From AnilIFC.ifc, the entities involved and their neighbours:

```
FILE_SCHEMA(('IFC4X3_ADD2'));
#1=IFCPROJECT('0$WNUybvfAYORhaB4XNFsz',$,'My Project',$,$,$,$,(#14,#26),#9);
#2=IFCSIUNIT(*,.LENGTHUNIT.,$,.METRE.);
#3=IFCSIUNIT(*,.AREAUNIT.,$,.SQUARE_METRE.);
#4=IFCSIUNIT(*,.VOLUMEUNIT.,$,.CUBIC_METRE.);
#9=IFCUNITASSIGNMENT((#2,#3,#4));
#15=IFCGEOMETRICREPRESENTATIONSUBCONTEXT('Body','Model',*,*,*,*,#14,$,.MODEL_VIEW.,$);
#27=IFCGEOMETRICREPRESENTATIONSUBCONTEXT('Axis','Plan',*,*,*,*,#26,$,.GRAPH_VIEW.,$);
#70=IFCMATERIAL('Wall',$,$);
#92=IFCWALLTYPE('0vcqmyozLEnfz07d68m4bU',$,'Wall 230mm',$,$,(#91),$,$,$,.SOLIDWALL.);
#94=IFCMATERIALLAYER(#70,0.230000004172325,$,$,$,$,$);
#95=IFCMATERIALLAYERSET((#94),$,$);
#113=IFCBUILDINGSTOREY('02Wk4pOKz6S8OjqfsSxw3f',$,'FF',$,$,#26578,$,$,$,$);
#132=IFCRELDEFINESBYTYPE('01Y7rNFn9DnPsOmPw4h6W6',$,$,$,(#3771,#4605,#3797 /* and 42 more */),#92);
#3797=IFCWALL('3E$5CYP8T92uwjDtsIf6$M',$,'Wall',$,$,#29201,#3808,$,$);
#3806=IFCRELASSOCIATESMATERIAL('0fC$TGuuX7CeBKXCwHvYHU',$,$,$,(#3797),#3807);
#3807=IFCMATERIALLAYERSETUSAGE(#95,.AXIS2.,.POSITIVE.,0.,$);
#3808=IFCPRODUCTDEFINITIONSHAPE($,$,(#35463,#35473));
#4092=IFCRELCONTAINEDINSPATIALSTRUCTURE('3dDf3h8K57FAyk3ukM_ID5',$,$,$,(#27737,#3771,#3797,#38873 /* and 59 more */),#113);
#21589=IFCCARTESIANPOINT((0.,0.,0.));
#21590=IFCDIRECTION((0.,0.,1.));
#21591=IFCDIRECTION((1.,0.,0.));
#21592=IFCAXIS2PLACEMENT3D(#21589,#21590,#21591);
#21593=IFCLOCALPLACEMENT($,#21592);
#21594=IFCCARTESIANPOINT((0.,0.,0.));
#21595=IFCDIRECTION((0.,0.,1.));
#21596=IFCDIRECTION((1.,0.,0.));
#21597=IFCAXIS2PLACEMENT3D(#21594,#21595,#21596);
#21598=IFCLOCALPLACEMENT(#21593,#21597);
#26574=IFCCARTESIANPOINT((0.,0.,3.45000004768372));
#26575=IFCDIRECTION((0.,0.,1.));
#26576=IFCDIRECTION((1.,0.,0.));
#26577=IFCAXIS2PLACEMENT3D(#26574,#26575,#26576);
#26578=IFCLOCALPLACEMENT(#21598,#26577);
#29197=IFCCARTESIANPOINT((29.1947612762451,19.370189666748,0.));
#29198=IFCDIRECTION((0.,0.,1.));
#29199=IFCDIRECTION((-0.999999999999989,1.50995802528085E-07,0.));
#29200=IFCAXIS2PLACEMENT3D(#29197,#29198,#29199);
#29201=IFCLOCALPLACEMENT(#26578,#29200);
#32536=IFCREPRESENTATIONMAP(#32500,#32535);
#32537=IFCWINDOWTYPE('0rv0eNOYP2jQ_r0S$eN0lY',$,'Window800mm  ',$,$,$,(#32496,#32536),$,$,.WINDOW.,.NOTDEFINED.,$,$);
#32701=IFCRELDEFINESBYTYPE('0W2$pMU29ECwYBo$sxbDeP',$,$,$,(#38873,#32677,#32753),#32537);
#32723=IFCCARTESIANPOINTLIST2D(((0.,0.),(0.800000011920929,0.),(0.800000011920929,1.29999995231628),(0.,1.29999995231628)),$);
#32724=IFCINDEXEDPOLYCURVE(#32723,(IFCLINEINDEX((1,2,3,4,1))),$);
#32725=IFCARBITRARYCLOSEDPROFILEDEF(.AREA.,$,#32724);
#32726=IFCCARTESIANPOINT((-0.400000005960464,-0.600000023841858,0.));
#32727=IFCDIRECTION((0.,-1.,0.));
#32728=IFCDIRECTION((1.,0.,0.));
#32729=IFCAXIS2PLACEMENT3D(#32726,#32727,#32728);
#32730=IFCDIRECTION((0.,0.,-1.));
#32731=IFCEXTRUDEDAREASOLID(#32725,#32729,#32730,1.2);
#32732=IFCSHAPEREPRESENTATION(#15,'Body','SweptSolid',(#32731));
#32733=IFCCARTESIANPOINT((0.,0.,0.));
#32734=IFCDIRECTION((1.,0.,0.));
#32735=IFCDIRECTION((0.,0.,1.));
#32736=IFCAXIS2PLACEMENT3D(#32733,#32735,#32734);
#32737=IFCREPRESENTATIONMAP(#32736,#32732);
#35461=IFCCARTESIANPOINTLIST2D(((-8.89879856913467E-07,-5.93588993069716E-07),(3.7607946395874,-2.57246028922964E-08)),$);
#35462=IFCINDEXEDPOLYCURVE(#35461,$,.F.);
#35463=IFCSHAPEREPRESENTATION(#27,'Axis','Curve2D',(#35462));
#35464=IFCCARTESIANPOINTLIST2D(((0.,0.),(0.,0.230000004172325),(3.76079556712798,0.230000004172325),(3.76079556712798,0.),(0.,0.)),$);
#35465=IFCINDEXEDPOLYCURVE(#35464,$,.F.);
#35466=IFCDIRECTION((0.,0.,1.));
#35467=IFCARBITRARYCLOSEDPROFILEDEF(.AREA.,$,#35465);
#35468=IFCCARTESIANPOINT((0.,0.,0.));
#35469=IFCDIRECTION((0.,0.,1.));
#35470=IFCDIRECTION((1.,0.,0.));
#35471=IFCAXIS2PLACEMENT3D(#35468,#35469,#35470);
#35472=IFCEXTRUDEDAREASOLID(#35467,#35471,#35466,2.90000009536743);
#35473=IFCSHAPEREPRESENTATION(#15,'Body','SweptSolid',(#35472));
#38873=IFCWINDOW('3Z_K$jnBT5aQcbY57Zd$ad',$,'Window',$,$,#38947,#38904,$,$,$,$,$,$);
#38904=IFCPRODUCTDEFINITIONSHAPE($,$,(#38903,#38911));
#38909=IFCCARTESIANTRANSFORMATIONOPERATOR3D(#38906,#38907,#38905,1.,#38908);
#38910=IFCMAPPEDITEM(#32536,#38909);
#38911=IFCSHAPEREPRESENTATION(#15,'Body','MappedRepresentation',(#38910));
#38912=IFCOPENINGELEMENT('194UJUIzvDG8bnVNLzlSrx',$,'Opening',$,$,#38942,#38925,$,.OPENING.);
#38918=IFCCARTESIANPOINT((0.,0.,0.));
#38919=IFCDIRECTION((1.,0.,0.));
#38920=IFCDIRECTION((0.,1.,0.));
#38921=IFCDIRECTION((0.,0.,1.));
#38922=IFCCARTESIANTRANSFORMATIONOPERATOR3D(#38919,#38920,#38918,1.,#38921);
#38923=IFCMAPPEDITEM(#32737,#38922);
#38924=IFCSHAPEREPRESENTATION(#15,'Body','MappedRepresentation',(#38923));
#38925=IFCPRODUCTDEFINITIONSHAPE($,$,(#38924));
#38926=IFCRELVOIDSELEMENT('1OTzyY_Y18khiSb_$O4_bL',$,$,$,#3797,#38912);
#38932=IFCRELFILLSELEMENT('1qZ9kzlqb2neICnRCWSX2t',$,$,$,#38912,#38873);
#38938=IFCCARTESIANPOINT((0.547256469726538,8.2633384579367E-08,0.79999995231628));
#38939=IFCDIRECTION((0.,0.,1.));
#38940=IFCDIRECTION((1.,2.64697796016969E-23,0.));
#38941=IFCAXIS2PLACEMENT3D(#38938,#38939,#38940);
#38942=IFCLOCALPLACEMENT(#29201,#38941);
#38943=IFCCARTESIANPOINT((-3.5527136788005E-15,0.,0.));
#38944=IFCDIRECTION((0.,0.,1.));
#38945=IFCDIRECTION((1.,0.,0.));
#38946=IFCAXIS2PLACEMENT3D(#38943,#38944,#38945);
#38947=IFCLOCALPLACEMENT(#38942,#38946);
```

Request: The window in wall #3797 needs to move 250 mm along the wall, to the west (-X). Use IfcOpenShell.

```python
import ifcopenshell
import ifcopenshell.api.geometry
import ifcopenshell.util.placement
import ifcopenshell.util.unit

model = ifcopenshell.open("AnilIFC.ifc")
unit_scale = ifcopenshell.util.unit.calculate_unit_scale(model)

window = model.by_guid("3Z_K$jnBT5aQcbY57Zd$ad")
opening = window.FillsVoids[0].RelatingOpeningElement
wall = opening.VoidsElements[0].RelatingBuildingElement

wall_matrix = ifcopenshell.util.placement.get_local_placement(wall.ObjectPlacement)
shift = wall_matrix[:3, 0] * 0.25 / unit_scale
before = ifcopenshell.util.placement.get_local_placement(window.ObjectPlacement)[:3, 3].copy()

# The window is placed relative to its opening, so it follows when the opening moves.
matrix = ifcopenshell.util.placement.get_local_placement(opening.ObjectPlacement)
matrix[:3, 3] += shift
ifcopenshell.api.geometry.edit_object_placement(
    model, product=opening, matrix=matrix, is_si=False, should_transform_children=True
)

after = ifcopenshell.util.placement.get_local_placement(window.ObjectPlacement)[:3, 3]
print("window moved by", (after - before).round(3) + 0.0)

model.write("AnilIFC_v2.ifc")
```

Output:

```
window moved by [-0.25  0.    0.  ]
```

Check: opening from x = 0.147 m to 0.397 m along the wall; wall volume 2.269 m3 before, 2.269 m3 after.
